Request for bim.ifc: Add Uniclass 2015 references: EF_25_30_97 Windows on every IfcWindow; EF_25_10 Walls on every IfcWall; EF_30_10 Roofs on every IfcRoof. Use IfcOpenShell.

First a look at what the model holds.

```python
import ifcopenshell

model = ifcopenshell.open("bim.ifc")
print(model.schema)
print("classifications:", [c.Name for c in model.by_type("IfcClassification")])
for ifc_class in ("IfcDoor", "IfcRoof", "IfcStair", "IfcWall", "IfcWindow"):
    print(ifc_class, len(model.by_type(ifc_class)))
```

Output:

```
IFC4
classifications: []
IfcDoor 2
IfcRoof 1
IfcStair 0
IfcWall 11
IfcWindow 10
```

```python
import ifcopenshell
import ifcopenshell.api.classification

model = ifcopenshell.open("bim.ifc")

system = ifcopenshell.api.classification.add_classification(model, classification="Uniclass 2015")

codes = {
    "IfcWindow": ("EF_25_30_97", "Windows"),
    "IfcWall": ("EF_25_10", "Walls"),
    "IfcRoof": ("EF_30_10", "Roofs"),
}
for ifc_class, (code, name) in codes.items():
    products = model.by_type(ifc_class)
    ifcopenshell.api.classification.add_reference(
        model, products=products, classification=system, identification=code, name=name
    )
    print(code, len(products))

model.write("bim_v2.ifc")
```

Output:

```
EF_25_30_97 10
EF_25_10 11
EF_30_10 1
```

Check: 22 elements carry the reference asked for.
